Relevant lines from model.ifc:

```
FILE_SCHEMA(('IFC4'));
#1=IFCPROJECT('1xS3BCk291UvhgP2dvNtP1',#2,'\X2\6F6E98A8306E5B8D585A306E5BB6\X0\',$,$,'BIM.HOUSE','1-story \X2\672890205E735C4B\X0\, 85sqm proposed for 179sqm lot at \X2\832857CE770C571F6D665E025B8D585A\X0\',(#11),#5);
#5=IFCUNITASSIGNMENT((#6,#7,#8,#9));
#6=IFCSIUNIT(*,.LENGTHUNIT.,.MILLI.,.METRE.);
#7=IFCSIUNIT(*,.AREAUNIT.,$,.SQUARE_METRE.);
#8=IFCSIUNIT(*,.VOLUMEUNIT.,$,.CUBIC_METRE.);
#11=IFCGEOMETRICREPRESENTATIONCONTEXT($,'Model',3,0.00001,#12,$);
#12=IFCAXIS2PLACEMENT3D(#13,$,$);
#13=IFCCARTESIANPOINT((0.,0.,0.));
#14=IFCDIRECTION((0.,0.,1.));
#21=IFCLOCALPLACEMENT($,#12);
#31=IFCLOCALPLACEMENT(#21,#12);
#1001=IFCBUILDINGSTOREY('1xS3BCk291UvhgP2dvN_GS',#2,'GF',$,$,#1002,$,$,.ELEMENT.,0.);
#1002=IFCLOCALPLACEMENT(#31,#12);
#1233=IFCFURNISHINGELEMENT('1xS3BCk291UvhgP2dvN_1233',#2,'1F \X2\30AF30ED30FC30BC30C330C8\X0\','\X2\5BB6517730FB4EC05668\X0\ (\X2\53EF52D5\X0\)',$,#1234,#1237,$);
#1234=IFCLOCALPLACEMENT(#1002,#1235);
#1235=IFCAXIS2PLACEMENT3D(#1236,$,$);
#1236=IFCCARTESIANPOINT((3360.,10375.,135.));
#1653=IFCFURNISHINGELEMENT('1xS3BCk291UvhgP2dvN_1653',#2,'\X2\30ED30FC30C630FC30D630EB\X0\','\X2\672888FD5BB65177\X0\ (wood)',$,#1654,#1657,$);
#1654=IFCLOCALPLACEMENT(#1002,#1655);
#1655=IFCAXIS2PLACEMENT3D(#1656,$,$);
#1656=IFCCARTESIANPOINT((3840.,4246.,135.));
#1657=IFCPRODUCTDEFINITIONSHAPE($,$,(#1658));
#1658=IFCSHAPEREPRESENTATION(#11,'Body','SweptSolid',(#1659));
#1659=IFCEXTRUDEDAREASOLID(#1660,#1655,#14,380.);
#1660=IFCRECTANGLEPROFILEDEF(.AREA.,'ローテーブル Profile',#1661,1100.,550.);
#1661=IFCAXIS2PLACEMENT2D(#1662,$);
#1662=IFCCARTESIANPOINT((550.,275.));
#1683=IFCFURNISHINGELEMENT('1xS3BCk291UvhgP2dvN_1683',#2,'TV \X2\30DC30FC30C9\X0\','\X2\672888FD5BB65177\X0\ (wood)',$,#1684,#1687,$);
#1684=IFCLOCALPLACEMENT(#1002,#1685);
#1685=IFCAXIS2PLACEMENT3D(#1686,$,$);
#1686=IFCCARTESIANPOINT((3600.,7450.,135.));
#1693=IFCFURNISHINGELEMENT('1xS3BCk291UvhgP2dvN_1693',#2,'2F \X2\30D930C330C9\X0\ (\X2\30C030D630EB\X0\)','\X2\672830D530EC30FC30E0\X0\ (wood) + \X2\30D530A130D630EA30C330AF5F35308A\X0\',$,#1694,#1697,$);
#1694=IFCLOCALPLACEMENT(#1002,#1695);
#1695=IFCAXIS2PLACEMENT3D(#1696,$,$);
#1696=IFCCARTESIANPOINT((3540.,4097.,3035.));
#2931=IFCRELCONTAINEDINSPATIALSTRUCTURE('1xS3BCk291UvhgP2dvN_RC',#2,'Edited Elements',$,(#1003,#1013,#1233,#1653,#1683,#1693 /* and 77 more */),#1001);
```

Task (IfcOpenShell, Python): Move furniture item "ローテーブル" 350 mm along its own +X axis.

```python
import ifcopenshell
import ifcopenshell.api.geometry
import ifcopenshell.util.placement

model = ifcopenshell.open("model.ifc")

item = model.by_guid("1xS3BCk291UvhgP2dvN_1653")
matrix = ifcopenshell.util.placement.get_local_placement(item.ObjectPlacement)
matrix[:3, 3] += matrix[:3, 0] * 350.0
ifcopenshell.api.geometry.edit_object_placement(model, product=item, matrix=matrix, is_si=False)

print(ifcopenshell.util.placement.get_local_placement(item.ObjectPlacement).round(3) + 0.0)

model.write("model_updated.ifc")
```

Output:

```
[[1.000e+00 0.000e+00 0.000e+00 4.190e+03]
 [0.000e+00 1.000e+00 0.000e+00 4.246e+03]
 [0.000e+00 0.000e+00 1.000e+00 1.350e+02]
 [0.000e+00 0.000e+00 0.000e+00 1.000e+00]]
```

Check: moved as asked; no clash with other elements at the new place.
